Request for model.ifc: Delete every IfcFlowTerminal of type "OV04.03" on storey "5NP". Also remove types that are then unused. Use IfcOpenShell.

First a look at what the model holds.

```python
import ifcopenshell
import ifcopenshell.util.element

model = ifcopenshell.open("model.ifc")
print(model.schema)
storey = next(s for s in model.by_type("IfcBuildingStorey") if s.Name == "5NP")
terminals = [e for e in ifcopenshell.util.element.get_decomposition(storey) if e.is_a("IfcFlowTerminal")]
seen = {}
for e in terminals:
    element_type = ifcopenshell.util.element.get_type(e)
    name = element_type.Name if element_type not in (None, e) else None
    seen[name] = seen.get(name, 0) + 1
for name, count in sorted(seen.items(), key=str):
    print(count, "x", name)
```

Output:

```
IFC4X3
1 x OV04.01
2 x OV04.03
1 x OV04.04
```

```python
import ifcopenshell
import ifcopenshell.api.root
import ifcopenshell.util.element

model = ifcopenshell.open("model.ifc")

storey = next(s for s in model.by_type("IfcBuildingStorey") if s.Name == "5NP")
terminals = [e for e in ifcopenshell.util.element.get_decomposition(storey) if e.is_a("IfcFlowTerminal")]
targets = [e for e in terminals if (t := ifcopenshell.util.element.get_type(e)) not in (None, e) and t.Name == "OV04.03"]
types = {ifcopenshell.util.element.get_type(e) for e in targets} - {None, *targets}

for e in targets:
    ifcopenshell.api.root.remove_product(model, product=e)
print(len(targets), "removed")

unused = [t for t in types if not ifcopenshell.util.element.get_types(t)]
for t in unused:
    ifcopenshell.api.root.remove_product(model, product=t)
print(len(unused), "unused types removed")

model.write("model-out.ifc")
```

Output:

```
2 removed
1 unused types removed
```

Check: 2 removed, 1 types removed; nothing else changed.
